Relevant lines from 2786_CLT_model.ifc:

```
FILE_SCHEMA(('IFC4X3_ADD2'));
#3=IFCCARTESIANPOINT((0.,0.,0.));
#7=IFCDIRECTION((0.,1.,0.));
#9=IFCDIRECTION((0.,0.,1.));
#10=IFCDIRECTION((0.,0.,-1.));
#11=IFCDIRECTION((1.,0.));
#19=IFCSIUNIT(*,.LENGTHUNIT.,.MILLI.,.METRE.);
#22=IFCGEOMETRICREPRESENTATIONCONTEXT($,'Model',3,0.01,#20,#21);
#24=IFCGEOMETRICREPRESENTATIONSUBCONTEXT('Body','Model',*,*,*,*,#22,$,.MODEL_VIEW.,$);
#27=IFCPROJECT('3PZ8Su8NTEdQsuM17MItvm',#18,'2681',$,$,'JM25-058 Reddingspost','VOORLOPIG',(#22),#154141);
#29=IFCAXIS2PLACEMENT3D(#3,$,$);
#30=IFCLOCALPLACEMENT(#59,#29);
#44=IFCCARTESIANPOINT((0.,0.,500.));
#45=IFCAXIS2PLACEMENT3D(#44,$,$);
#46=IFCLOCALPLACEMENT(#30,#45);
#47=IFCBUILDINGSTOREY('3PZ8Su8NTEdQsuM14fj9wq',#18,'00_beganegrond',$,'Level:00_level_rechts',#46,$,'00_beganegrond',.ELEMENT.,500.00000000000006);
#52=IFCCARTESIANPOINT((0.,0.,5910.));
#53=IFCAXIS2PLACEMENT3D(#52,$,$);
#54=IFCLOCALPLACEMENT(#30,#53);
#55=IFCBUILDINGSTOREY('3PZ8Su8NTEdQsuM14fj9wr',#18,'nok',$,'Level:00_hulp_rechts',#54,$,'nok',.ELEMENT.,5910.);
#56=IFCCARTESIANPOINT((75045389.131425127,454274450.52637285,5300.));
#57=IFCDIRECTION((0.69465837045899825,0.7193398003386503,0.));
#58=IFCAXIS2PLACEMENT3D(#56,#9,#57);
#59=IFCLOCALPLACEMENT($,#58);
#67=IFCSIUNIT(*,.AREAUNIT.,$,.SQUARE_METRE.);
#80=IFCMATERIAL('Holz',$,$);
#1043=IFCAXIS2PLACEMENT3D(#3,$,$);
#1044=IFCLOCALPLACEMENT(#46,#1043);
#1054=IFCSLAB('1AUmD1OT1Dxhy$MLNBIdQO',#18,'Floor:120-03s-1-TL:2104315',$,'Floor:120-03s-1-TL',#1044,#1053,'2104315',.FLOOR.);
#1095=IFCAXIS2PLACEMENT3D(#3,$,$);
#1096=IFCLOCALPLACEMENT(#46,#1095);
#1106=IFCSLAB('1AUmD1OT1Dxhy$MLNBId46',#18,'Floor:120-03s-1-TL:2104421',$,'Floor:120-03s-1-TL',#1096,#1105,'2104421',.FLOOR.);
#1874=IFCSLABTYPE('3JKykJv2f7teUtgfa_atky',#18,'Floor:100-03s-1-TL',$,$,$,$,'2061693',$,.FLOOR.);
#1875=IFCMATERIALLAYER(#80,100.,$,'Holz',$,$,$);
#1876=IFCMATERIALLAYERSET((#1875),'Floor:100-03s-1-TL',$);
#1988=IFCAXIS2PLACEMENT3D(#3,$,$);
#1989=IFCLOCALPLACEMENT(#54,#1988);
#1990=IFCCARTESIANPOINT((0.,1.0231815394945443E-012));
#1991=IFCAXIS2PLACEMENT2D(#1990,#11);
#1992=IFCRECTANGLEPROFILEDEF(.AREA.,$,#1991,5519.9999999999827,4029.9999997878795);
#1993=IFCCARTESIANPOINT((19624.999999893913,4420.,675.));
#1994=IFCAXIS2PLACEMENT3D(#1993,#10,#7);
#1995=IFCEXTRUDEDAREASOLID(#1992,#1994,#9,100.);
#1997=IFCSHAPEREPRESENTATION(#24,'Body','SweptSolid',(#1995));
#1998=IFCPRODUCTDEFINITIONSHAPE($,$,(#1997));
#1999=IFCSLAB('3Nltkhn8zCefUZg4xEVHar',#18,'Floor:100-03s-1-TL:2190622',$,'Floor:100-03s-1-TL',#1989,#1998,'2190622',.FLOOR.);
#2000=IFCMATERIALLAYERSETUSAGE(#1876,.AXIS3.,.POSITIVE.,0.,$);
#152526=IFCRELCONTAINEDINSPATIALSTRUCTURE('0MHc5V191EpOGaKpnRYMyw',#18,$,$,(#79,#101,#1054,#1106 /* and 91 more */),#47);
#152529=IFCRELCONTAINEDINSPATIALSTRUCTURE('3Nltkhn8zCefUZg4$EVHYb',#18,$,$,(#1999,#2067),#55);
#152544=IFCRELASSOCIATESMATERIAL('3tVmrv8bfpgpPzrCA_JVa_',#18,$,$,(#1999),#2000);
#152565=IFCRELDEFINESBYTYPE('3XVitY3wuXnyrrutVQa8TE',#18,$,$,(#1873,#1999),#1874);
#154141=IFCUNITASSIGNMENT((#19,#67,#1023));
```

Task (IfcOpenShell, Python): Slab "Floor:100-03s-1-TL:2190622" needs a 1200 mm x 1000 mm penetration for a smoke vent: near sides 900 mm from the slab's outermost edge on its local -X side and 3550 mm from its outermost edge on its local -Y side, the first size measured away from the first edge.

```python
import numpy as np
import ifcopenshell
import ifcopenshell.api.feature
import ifcopenshell.api.geometry
import ifcopenshell.api.root
import ifcopenshell.geom
import ifcopenshell.util.placement
import ifcopenshell.util.representation
import ifcopenshell.util.shape
import ifcopenshell.util.unit

model = ifcopenshell.open("2786_CLT_model.ifc")
unit_scale = ifcopenshell.util.unit.calculate_unit_scale(model)
settings = ifcopenshell.geom.settings()


def volume(element):
    """Net volume in cubic metres, openings subtracted."""
    shape = ifcopenshell.geom.create_shape(settings, element)
    return ifcopenshell.util.shape.get_volume(shape.geometry)


slab = model.by_guid("3Nltkhn8zCefUZg4xEVHar")
before = volume(slab)

# Extent in the slab's own axes, in metres. The edges named are its -X and -Y sides.
slab_shape = ifcopenshell.geom.create_shape(settings, slab)
vertices = ifcopenshell.util.shape.get_vertices(slab_shape.geometry)
x_min, y_min, bottom = vertices.min(axis=0)
top = vertices[:, 2].max()

opening = ifcopenshell.api.root.create_entity(model, ifc_class="IfcOpeningElement", name="Smoke vent opening", predefined_type="OPENING")
context = ifcopenshell.util.representation.get_context(model, "Model", "Body", "MODEL_VIEW")
width, depth = 1.2, 1
outline = [(0.0, 0.0), (width, 0.0), (width, depth), (0.0, depth), (0.0, 0.0)]
# Overshoot both faces by 50 mm so the cut is clean.
shape = ifcopenshell.api.geometry.add_slab_representation(
    model, context=context, depth=top - bottom + 0.1, polyline=outline
)
ifcopenshell.api.geometry.assign_representation(model, product=opening, representation=shape)

matrix = ifcopenshell.util.placement.get_local_placement(slab.ObjectPlacement)
matrix[:, 3] = matrix @ np.append(np.array([x_min + 0.9, y_min + 3.55, bottom - 0.05]) / unit_scale, 1.0)
ifcopenshell.api.geometry.edit_object_placement(model, product=opening, matrix=matrix, is_si=False)
ifcopenshell.api.feature.add_feature(model, feature=opening, element=slab)

after = volume(slab)

print(f"slab volume {before:.3f} -> {after:.3f} m3")

model.write("2786_CLT_model-out.ifc")
```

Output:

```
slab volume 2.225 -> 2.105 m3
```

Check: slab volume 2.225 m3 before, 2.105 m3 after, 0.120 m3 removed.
